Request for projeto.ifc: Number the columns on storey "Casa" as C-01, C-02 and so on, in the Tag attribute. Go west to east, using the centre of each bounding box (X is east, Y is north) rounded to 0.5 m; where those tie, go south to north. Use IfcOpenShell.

First a look at what the model holds.

```python
import ifcopenshell
import ifcopenshell.util.element
import ifcopenshell.util.placement

model = ifcopenshell.open("projeto.ifc")
print(model.schema)
storey = next(s for s in model.by_type("IfcBuildingStorey") if s.Name == "Casa")
columns = [e for e in ifcopenshell.util.element.get_decomposition(storey) if e.is_a("IfcColumn")]
for e in sorted(columns, key=lambda e: e.id()):
    origin = ifcopenshell.util.placement.get_local_placement(e.ObjectPlacement)[:3, 3]
    print(e.id(), e.Tag, e.Name, origin.round(2) + 0.0, sep=" | ")
```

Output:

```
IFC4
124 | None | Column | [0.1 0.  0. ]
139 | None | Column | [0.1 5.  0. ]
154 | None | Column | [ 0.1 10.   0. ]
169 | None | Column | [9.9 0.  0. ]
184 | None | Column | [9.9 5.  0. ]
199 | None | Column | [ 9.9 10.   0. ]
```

```python
import ifcopenshell
import ifcopenshell.geom
import ifcopenshell.util.element
import ifcopenshell.util.shape

model = ifcopenshell.open("projeto.ifc")
settings = ifcopenshell.geom.settings()
settings.set("use-world-coords", True)


def centre(element):
    shape = ifcopenshell.geom.create_shape(settings, element)
    return ifcopenshell.util.shape.get_bbox_centroid(shape.geometry)


storey = next(s for s in model.by_type("IfcBuildingStorey") if s.Name == "Casa")
columns = [e for e in ifcopenshell.util.element.get_decomposition(storey) if e.is_a("IfcColumn")]

# Insertion points can sit at a corner or the storey origin, so sort by the geometry (in metres).
centres = {e: centre(e) for e in columns}
columns.sort(key=lambda e: (round(centres[e][0] / 0.5), centres[e][1]))

for i, e in enumerate(columns, start=1):
    number = f"C-{i:02d}"
    e.Tag = number
    print(e.id(), number)

model.write("projeto_updated.ifc")
```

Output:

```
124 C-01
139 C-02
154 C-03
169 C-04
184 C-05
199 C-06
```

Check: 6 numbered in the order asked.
